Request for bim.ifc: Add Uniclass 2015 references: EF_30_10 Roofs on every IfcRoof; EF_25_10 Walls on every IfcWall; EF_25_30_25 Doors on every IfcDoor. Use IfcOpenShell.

First a look at what the model holds.

```python
import ifcopenshell

model = ifcopenshell.open("bim.ifc")
print(model.schema)
print("classifications:", [c.Name for c in model.by_type("IfcClassification")])
for ifc_class in ("IfcDoor", "IfcRoof", "IfcStair", "IfcWall", "IfcWindow"):
    print(ifc_class, len(model.by_type(ifc_class)))
```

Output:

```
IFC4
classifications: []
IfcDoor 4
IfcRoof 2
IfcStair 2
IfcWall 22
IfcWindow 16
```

```python
import ifcopenshell
import ifcopenshell.api.classification

model = ifcopenshell.open("bim.ifc")

system = ifcopenshell.api.classification.add_classification(model, classification="Uniclass 2015")

codes = {
    "IfcRoof": ("EF_30_10", "Roofs"),
    "IfcWall": ("EF_25_10", "Walls"),
    "IfcDoor": ("EF_25_30_25", "Doors"),
}
for ifc_class, (code, name) in codes.items():
    products = model.by_type(ifc_class)
    ifcopenshell.api.classification.add_reference(
        model, products=products, classification=system, identification=code, name=name
    )
    print(code, len(products))

model.write("bim_updated.ifc")
```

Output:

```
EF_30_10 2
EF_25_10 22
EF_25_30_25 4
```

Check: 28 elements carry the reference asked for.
